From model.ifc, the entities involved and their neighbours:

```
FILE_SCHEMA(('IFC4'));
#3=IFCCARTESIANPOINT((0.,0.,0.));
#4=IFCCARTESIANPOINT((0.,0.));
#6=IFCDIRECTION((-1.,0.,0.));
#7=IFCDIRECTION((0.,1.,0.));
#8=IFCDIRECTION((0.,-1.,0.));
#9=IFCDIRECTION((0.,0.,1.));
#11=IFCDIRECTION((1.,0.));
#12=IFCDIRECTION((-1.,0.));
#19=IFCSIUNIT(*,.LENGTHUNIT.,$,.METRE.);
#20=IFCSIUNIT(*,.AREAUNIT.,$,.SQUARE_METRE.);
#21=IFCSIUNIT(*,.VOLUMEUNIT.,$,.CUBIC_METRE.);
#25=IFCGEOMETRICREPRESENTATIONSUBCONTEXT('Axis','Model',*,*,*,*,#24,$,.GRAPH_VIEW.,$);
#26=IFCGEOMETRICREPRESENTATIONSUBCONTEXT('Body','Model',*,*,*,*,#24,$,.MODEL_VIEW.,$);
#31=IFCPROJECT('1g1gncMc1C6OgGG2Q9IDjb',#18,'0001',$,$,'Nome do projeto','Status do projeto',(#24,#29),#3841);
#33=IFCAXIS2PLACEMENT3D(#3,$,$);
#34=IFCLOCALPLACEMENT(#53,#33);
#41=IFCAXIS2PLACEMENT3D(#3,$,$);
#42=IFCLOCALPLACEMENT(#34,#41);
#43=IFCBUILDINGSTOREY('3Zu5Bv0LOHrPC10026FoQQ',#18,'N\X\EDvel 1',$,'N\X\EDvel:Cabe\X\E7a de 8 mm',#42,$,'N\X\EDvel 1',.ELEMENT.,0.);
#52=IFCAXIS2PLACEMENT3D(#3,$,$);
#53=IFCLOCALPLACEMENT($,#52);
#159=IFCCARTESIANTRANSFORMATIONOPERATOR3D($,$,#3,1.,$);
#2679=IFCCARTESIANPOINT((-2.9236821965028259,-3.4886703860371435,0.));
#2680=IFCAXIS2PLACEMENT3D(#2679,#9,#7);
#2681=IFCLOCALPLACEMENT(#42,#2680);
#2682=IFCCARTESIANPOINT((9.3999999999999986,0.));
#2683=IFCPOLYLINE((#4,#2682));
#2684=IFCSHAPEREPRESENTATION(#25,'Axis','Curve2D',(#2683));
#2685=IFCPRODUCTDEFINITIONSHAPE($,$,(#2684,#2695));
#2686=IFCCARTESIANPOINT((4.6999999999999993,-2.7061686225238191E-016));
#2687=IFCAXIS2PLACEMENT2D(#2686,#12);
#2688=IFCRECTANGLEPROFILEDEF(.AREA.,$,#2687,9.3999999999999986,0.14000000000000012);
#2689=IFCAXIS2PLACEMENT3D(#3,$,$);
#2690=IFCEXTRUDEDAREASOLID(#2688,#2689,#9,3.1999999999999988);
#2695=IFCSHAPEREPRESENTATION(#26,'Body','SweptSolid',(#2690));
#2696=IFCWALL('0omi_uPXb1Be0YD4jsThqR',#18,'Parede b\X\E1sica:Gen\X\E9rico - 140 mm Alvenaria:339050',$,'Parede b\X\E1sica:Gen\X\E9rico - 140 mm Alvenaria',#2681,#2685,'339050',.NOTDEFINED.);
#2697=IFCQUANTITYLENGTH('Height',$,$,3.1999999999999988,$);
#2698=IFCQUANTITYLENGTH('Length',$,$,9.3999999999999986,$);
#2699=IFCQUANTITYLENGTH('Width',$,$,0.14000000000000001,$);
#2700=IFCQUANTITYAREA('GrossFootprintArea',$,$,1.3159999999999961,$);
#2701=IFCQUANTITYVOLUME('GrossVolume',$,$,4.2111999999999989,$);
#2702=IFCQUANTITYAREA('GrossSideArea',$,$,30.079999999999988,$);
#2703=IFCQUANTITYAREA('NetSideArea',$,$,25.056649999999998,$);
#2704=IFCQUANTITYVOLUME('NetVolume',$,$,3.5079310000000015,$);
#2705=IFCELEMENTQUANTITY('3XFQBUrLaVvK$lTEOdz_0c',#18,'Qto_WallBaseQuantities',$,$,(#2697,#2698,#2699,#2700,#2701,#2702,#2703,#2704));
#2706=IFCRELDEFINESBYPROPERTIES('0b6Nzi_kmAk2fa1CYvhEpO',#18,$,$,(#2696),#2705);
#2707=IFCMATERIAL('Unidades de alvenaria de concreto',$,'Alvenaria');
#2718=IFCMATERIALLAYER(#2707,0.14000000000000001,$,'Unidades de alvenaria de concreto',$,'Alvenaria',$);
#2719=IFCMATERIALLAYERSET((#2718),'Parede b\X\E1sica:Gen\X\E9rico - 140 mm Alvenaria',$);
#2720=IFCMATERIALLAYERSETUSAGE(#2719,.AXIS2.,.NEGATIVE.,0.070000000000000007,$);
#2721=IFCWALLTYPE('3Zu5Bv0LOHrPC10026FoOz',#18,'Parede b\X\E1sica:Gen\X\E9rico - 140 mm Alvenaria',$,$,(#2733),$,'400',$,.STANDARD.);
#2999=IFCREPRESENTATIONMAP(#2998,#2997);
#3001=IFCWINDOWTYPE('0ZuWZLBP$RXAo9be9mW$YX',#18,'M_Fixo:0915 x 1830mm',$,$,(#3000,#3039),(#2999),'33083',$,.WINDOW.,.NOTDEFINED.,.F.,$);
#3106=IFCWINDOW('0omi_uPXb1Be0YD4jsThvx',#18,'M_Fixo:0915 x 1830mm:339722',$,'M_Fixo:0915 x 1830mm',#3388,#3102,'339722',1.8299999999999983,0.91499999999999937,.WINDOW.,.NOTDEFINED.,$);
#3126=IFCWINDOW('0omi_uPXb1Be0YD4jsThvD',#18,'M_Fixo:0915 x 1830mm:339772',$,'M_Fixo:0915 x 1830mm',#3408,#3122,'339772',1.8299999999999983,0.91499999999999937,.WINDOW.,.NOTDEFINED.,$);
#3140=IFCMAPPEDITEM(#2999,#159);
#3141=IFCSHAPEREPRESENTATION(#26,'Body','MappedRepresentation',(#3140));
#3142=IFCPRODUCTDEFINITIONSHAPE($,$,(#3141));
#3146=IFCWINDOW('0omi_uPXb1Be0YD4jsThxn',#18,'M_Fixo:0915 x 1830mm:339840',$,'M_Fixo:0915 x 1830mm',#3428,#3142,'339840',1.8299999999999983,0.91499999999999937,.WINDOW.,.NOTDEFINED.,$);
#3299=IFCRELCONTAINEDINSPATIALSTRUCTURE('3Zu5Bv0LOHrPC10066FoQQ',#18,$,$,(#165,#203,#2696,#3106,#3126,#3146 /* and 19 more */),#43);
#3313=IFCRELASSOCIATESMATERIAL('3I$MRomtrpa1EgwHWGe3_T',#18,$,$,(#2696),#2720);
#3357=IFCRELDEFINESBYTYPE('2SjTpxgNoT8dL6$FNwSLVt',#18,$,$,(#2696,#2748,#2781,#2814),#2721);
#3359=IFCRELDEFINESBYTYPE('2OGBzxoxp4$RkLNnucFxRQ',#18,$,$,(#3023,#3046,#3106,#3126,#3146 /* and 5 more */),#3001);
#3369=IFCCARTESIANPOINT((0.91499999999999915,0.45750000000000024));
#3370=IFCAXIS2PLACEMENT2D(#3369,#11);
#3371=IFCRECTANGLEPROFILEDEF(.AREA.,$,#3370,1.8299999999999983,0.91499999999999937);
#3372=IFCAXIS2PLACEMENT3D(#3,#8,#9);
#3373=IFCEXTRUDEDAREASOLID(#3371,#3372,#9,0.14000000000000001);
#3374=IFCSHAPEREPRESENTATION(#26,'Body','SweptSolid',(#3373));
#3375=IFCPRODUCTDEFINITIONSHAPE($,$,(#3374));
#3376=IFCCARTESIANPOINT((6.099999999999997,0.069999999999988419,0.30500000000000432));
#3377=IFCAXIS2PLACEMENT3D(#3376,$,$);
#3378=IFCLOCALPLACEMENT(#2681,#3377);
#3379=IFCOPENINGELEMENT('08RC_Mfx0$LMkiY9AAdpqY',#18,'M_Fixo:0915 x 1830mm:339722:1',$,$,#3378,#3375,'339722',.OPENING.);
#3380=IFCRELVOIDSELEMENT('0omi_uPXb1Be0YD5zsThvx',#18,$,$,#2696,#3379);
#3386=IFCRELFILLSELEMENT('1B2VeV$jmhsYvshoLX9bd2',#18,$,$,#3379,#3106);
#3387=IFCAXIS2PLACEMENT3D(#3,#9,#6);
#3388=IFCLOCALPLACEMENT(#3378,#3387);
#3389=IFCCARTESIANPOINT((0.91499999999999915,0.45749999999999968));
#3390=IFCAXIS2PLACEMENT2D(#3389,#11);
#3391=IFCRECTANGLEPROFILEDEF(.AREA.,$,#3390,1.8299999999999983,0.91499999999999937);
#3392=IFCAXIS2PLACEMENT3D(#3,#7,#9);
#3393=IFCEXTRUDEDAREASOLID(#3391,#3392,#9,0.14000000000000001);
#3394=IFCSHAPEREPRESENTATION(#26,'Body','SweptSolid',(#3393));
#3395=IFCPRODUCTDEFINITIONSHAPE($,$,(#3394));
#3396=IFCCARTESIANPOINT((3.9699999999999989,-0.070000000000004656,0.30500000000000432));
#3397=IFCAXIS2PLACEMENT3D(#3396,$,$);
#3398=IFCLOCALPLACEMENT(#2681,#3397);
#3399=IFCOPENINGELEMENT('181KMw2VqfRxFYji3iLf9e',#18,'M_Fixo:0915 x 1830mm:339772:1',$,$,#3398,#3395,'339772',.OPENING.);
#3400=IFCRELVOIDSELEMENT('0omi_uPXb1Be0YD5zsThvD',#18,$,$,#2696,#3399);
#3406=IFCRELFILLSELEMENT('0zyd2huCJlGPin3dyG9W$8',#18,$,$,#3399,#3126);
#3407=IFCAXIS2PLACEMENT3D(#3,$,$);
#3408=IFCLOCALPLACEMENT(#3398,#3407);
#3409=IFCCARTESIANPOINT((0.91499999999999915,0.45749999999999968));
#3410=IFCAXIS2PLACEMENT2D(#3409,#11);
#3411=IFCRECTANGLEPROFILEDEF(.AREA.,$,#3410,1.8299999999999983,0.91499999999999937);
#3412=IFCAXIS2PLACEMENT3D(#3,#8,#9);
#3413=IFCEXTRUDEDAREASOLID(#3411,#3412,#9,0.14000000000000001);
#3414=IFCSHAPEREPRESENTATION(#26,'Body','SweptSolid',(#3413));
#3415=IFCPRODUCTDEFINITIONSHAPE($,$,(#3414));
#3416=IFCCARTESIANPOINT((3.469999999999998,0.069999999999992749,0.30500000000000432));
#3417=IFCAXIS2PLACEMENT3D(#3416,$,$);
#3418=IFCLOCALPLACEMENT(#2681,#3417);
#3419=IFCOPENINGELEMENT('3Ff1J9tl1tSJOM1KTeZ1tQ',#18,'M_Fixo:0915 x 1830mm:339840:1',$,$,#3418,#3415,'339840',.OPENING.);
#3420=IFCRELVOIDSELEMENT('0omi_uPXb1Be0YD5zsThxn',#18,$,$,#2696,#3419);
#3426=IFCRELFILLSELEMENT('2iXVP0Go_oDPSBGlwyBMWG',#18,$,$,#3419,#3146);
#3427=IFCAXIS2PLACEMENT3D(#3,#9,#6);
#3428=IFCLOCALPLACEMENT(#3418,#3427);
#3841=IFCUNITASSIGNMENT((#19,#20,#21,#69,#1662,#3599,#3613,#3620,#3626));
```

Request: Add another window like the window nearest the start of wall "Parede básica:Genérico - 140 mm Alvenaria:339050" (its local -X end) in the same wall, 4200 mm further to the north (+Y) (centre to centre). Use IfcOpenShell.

```python
import ifcopenshell
import ifcopenshell.api.feature
import ifcopenshell.api.geometry
import ifcopenshell.api.pset
import ifcopenshell.api.root
import ifcopenshell.geom
import ifcopenshell.util.element
import ifcopenshell.util.placement
import ifcopenshell.util.shape
import ifcopenshell.util.unit

model = ifcopenshell.open("model.ifc")
unit_scale = ifcopenshell.util.unit.calculate_unit_scale(model)
area_scale = ifcopenshell.util.unit.calculate_unit_scale(model, "AREAUNIT")
volume_scale = ifcopenshell.util.unit.calculate_unit_scale(model, "VOLUMEUNIT")
settings = ifcopenshell.geom.settings()


def volume(element):
    """Net volume in cubic metres, openings subtracted."""
    shape = ifcopenshell.geom.create_shape(settings, element)
    return ifcopenshell.util.shape.get_volume(shape.geometry)


def reuse_history(source, copy):
    """copy_class also copies each property set's owner history, people and application; keep the originals."""
    for rel in copy.IsDefinedBy:
        if rel.is_a("IfcRelDefinesByProperties") and (history := rel.RelatingPropertyDefinition.OwnerHistory):
            rel.RelatingPropertyDefinition.OwnerHistory = source.OwnerHistory
            ifcopenshell.util.element.remove_deep2(model, history)


window = model.by_guid("0omi_uPXb1Be0YD4jsThxn")
opening = window.FillsVoids[0].RelatingOpeningElement
wall = opening.VoidsElements[0].RelatingBuildingElement
before = volume(wall)
shift = ifcopenshell.util.placement.get_local_placement(wall.ObjectPlacement)[:3, 0] * 4.2 / unit_scale

# copy_class copies the void relationship, type, container and properties, but no geometry.
new_opening = ifcopenshell.api.root.copy_class(model, product=opening)
new_opening.Representation = ifcopenshell.util.element.copy_deep(
    model, opening.Representation, exclude=["IfcGeometricRepresentationContext", "IfcRepresentationMap"]
)
new_opening.Name = "M_Fixo:0915 x 1830mm"
new_opening.Tag = None
reuse_history(opening, new_opening)
new_window = ifcopenshell.api.root.copy_class(model, product=window)
new_window.Representation = ifcopenshell.util.element.copy_deep(
    model, window.Representation, exclude=["IfcGeometricRepresentationContext", "IfcRepresentationMap"]
)
new_window.Name = "M_Fixo:0915 x 1830mm"
new_window.Tag = None
reuse_history(window, new_window)
ifcopenshell.api.feature.add_filling(model, opening=new_opening, element=new_window)

for old, new in ((opening, new_opening), (window, new_window)):
    matrix = ifcopenshell.util.placement.get_local_placement(old.ObjectPlacement)
    matrix[:3, 3] += shift
    ifcopenshell.api.geometry.edit_object_placement(model, product=new, matrix=matrix, is_si=False)

after = volume(wall)
thickness = 0.14  # wall thickness in metres

# Update the wall's stored quantities.
qto = model.by_id(ifcopenshell.util.element.get_pset(wall, "Qto_WallBaseQuantities", should_inherit=False)["id"])
ifcopenshell.api.pset.edit_qto(model, qto=qto, properties={
    "NetSideArea": after / thickness / area_scale,
    "NetVolume": after / volume_scale,
})

print(f"wall volume {before:.3f} -> {after:.3f} m3")

model.write("model_edited.ifc")
```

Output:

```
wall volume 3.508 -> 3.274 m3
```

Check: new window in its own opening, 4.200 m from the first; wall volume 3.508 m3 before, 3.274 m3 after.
